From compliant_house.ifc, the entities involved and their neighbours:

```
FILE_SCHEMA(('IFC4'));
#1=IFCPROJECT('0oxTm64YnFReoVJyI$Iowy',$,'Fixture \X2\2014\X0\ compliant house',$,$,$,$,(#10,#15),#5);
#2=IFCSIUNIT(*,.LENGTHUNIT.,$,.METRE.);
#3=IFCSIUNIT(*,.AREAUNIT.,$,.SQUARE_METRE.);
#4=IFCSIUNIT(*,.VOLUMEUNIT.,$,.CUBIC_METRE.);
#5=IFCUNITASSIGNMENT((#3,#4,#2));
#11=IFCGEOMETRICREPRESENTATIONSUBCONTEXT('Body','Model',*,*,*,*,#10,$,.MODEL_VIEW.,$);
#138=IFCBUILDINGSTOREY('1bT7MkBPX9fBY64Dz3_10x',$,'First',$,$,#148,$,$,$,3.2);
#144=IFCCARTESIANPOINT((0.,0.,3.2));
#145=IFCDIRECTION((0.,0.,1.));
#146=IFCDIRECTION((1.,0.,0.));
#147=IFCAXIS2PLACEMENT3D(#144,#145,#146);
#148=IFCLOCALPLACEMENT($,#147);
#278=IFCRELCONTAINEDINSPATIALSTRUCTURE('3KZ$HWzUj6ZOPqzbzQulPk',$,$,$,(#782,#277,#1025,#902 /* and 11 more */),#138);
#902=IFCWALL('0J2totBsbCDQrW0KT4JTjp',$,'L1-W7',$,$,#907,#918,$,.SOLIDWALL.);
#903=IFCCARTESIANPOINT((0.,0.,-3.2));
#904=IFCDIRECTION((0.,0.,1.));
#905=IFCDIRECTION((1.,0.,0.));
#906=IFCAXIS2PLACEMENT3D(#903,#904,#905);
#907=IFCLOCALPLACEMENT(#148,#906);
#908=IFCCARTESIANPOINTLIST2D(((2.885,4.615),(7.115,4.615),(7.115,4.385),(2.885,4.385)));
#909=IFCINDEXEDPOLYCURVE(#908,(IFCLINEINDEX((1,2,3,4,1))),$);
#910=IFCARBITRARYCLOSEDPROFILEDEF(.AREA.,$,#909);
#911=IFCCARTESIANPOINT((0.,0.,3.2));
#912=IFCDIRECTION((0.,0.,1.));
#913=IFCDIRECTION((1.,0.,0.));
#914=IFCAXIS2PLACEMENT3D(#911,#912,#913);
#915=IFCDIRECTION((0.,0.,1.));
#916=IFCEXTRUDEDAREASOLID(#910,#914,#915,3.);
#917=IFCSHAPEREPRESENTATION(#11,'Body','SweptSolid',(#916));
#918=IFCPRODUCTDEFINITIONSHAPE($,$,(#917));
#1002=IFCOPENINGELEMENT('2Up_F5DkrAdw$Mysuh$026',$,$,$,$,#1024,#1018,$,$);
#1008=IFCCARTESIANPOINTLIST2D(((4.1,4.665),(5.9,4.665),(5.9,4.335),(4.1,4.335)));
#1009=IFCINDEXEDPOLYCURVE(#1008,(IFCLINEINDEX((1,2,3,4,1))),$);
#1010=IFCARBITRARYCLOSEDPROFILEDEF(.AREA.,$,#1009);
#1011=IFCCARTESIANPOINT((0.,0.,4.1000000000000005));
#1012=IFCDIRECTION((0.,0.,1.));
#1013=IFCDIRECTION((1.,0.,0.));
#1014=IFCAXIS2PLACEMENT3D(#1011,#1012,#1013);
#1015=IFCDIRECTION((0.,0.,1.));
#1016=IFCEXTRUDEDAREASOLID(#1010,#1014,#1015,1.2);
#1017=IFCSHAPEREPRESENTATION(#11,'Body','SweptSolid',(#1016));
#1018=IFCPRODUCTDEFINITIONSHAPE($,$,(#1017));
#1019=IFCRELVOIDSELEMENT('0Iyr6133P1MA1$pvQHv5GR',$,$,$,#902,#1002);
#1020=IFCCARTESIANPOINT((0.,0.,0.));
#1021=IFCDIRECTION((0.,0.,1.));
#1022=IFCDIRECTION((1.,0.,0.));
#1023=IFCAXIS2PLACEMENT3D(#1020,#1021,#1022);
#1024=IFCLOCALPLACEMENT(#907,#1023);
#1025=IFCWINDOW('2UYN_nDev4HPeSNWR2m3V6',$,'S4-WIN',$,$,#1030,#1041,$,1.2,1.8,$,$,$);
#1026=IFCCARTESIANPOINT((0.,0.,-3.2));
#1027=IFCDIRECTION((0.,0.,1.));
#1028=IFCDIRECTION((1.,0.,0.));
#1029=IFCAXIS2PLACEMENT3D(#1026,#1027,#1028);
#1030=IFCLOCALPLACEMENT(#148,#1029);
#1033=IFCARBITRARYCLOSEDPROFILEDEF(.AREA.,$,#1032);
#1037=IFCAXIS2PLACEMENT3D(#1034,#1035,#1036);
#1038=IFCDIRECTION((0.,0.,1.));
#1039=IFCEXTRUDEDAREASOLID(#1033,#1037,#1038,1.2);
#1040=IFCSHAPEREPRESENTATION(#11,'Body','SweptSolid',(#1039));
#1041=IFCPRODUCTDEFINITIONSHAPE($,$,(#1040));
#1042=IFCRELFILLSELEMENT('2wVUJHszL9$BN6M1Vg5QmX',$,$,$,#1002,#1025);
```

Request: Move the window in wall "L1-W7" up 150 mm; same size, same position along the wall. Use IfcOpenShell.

```python
import numpy as np
import ifcopenshell
import ifcopenshell.api.geometry
import ifcopenshell.util.placement
import ifcopenshell.util.unit

model = ifcopenshell.open("compliant_house.ifc")
unit_scale = ifcopenshell.util.unit.calculate_unit_scale(model)

window = model.by_guid("2UYN_nDev4HPeSNWR2m3V6")
opening = window.FillsVoids[0].RelatingOpeningElement
dz = 0.15 / unit_scale

shift = np.array([0.0, 0.0, dz])
# The window is not placed relative to its opening, so move both.
for product in (opening, window):
    matrix = ifcopenshell.util.placement.get_local_placement(product.ObjectPlacement)
    matrix[:3, 3] += shift
    ifcopenshell.api.geometry.edit_object_placement(model, product=product, matrix=matrix, is_si=False)

print(f"moved by {dz * unit_scale:+.3f} m")

model.write("compliant_house_v2.ifc")
```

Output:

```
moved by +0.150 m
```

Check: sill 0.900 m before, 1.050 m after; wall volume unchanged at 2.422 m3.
